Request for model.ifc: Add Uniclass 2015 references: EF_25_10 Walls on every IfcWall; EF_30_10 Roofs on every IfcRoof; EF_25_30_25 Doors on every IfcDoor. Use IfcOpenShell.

First a look at what the model holds.

```python
import ifcopenshell

model = ifcopenshell.open("model.ifc")
print(model.schema)
print("classifications:", [c.Name for c in model.by_type("IfcClassification")])
for ifc_class in ("IfcDoor", "IfcRoof", "IfcStair", "IfcWall", "IfcWindow"):
    print(ifc_class, len(model.by_type(ifc_class)))
```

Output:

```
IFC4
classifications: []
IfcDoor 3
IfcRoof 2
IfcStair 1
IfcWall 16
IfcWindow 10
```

```python
import ifcopenshell
import ifcopenshell.api.classification

model = ifcopenshell.open("model.ifc")

system = ifcopenshell.api.classification.add_classification(model, classification="Uniclass 2015")

codes = {
    "IfcWall": ("EF_25_10", "Walls"),
    "IfcRoof": ("EF_30_10", "Roofs"),
    "IfcDoor": ("EF_25_30_25", "Doors"),
}
for ifc_class, (code, name) in codes.items():
    products = model.by_type(ifc_class)
    ifcopenshell.api.classification.add_reference(
        model, products=products, classification=system, identification=code, name=name
    )
    print(code, len(products))

model.write("model-out.ifc")
```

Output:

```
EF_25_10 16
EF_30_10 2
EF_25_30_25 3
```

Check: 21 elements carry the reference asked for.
